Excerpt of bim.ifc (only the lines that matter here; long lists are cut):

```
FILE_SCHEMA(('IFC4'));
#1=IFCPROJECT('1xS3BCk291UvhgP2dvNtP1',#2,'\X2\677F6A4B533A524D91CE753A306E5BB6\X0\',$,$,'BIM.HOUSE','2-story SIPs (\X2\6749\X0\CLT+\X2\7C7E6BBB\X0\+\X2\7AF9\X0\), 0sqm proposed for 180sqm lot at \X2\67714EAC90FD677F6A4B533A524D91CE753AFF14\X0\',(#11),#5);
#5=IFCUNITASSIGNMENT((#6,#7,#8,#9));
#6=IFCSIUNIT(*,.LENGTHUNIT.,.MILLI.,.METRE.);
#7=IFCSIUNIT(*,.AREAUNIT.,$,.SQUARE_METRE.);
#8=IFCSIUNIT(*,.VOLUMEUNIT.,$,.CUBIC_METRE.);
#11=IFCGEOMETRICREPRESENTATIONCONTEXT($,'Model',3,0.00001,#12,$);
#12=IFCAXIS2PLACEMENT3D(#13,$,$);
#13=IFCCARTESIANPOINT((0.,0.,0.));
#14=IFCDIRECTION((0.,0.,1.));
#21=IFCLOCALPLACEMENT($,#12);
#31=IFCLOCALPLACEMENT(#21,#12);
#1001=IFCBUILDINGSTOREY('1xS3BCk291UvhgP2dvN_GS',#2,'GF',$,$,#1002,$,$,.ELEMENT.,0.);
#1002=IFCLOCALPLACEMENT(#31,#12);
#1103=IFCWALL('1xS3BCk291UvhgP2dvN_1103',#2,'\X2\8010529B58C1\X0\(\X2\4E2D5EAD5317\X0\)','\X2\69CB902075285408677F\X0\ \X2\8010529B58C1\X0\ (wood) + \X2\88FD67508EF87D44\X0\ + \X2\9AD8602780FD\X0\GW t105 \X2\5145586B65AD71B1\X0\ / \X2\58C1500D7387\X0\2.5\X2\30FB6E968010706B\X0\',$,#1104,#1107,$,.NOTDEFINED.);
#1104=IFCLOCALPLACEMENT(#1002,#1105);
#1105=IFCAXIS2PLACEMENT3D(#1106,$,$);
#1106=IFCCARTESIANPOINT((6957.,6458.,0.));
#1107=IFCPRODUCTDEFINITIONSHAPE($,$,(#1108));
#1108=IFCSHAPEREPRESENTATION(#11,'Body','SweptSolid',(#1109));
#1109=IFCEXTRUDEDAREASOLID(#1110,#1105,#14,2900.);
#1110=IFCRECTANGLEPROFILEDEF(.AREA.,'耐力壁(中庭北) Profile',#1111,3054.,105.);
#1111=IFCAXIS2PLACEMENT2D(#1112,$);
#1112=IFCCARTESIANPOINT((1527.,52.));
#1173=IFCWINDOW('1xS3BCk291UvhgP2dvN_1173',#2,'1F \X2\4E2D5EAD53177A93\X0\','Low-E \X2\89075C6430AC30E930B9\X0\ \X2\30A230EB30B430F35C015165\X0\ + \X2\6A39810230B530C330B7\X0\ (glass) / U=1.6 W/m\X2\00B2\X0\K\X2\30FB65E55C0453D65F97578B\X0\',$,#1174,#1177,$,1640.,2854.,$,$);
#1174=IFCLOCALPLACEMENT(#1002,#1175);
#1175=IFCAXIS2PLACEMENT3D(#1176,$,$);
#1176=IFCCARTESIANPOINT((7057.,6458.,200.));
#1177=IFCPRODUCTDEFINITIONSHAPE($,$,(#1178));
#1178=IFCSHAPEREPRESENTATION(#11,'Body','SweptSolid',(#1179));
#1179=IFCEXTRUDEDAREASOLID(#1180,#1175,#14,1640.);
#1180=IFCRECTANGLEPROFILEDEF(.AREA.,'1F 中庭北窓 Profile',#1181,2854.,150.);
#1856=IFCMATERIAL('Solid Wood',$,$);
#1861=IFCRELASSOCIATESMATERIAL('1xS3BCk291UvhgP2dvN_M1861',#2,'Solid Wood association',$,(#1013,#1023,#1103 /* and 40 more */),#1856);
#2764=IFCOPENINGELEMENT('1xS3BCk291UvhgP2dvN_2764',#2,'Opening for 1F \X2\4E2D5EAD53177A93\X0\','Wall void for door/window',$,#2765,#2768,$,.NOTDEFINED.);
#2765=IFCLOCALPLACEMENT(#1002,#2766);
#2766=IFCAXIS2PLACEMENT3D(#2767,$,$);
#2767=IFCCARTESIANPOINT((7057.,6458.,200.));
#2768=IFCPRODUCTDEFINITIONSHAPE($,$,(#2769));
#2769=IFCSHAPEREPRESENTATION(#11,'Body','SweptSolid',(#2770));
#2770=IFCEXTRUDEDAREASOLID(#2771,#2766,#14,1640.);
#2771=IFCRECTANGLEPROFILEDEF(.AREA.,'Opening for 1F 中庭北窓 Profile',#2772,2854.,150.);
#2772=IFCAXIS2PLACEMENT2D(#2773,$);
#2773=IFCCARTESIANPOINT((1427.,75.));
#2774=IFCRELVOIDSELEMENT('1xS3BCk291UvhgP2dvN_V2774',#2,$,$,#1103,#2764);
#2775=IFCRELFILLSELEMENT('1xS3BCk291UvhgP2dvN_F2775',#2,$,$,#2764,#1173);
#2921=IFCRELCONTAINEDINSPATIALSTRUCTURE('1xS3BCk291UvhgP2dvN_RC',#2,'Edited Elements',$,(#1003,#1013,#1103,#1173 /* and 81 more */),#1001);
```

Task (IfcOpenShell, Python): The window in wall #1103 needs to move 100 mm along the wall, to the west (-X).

```python
import ifcopenshell
import ifcopenshell.api.geometry
import ifcopenshell.util.placement
import ifcopenshell.util.unit

model = ifcopenshell.open("bim.ifc")
unit_scale = ifcopenshell.util.unit.calculate_unit_scale(model)

window = model.by_id(1173)
opening = window.FillsVoids[0].RelatingOpeningElement
wall = opening.VoidsElements[0].RelatingBuildingElement

wall_matrix = ifcopenshell.util.placement.get_local_placement(wall.ObjectPlacement)
shift = wall_matrix[:3, 0] * -0.1 / unit_scale
before = ifcopenshell.util.placement.get_local_placement(window.ObjectPlacement)[:3, 3].copy()

# The window is not placed relative to its opening, so move both.
for product in (opening, window):
    matrix = ifcopenshell.util.placement.get_local_placement(product.ObjectPlacement)
    matrix[:3, 3] += shift
    ifcopenshell.api.geometry.edit_object_placement(model, product=product, matrix=matrix, is_si=False)

after = ifcopenshell.util.placement.get_local_placement(window.ObjectPlacement)[:3, 3]
print("window moved by", (after - before).round(3) + 0.0)

model.write("bim-out.ifc")
```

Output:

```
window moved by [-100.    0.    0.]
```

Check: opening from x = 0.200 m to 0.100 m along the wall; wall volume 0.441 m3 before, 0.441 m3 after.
